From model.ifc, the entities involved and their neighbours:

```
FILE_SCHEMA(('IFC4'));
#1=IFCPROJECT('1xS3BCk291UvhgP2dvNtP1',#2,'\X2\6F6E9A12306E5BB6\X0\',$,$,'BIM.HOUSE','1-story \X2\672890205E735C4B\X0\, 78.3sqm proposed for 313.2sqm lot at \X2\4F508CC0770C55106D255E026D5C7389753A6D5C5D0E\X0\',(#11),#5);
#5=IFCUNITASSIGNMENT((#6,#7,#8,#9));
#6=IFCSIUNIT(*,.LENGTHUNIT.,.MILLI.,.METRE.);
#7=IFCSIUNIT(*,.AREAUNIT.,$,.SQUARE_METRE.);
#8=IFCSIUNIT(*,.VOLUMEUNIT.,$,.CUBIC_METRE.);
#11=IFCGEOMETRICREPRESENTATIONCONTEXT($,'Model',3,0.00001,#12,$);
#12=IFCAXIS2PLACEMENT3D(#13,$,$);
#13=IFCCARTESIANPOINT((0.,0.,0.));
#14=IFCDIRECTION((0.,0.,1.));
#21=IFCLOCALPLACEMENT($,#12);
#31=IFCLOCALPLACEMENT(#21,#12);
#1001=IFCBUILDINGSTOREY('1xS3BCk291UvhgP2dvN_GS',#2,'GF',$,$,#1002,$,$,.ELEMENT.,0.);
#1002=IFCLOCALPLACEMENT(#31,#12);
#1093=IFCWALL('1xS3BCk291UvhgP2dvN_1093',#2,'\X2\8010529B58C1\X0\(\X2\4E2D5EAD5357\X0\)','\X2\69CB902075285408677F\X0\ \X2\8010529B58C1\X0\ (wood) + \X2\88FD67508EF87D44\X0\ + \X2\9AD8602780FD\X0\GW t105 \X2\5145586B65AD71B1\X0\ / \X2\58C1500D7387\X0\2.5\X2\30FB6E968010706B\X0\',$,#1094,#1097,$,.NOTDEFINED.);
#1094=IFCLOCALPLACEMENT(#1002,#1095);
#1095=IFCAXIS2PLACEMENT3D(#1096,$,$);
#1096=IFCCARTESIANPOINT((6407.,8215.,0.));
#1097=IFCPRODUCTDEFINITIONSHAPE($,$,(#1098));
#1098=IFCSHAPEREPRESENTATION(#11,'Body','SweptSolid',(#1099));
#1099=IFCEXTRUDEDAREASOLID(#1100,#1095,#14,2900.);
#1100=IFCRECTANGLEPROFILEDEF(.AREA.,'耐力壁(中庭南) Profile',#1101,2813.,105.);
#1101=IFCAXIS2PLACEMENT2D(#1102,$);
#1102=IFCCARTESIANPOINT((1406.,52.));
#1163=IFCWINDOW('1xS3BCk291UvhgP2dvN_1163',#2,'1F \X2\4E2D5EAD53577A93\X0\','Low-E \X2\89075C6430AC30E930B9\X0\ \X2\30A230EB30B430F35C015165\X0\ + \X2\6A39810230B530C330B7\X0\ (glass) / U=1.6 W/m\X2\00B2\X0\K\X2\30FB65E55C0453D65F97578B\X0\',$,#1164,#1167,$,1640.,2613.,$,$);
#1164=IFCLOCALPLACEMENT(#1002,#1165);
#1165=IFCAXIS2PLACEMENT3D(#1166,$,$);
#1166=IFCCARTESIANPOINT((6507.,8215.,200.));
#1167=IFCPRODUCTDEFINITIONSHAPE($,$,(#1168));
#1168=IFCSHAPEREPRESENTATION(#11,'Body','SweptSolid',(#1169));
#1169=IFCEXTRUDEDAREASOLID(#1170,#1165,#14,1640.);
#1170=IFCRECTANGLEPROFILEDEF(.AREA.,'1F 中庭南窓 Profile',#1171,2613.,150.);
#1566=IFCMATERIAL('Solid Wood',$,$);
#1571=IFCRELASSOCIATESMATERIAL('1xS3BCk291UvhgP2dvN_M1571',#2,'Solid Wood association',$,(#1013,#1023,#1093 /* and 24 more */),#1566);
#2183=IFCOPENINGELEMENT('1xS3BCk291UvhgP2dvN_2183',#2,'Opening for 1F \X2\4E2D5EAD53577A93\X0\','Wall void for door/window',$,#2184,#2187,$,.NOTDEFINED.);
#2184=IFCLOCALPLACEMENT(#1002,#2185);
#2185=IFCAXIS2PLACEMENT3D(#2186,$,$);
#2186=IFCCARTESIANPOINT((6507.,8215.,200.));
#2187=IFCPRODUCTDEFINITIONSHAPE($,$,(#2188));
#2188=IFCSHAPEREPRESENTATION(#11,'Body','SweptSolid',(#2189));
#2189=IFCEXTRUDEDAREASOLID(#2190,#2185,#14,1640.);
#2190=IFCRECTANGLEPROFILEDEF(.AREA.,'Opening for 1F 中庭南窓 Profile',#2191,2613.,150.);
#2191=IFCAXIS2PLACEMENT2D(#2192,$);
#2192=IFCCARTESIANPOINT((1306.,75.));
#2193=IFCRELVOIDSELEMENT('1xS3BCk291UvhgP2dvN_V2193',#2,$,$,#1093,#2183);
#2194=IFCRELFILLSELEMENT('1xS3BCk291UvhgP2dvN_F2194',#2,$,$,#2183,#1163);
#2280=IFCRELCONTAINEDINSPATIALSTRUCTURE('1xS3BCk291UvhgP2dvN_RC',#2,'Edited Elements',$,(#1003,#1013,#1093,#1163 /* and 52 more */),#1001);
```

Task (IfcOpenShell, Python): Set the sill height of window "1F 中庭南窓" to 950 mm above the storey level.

```python
import numpy as np
import ifcopenshell
import ifcopenshell.api.geometry
import ifcopenshell.geom
import ifcopenshell.util.element
import ifcopenshell.util.placement
import ifcopenshell.util.shape
import ifcopenshell.util.unit

model = ifcopenshell.open("model.ifc")
unit_scale = ifcopenshell.util.unit.calculate_unit_scale(model)

window = model.by_guid("1xS3BCk291UvhgP2dvN_1163")
opening = window.FillsVoids[0].RelatingOpeningElement
storey = ifcopenshell.util.element.get_container(window, ifc_class="IfcBuildingStorey")
level = ifcopenshell.util.placement.get_local_placement(storey.ObjectPlacement)[2, 3]

# The opening's origin need not be at the sill, so measure its lowest point.
shape = ifcopenshell.geom.create_shape(ifcopenshell.geom.settings(), opening)
bottom = ifcopenshell.util.shape.get_shape_bottom_elevation(shape, shape.geometry) / unit_scale
dz = level + 0.95 / unit_scale - bottom

shift = np.array([0.0, 0.0, dz])
# The window is not placed relative to its opening, so move both.
for product in (opening, window):
    matrix = ifcopenshell.util.placement.get_local_placement(product.ObjectPlacement)
    matrix[:3, 3] += shift
    ifcopenshell.api.geometry.edit_object_placement(model, product=product, matrix=matrix, is_si=False)

print(f"moved by {dz * unit_scale:+.3f} m")

model.write("model_v2.ifc")
```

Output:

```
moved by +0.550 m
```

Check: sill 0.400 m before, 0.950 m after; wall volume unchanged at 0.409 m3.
